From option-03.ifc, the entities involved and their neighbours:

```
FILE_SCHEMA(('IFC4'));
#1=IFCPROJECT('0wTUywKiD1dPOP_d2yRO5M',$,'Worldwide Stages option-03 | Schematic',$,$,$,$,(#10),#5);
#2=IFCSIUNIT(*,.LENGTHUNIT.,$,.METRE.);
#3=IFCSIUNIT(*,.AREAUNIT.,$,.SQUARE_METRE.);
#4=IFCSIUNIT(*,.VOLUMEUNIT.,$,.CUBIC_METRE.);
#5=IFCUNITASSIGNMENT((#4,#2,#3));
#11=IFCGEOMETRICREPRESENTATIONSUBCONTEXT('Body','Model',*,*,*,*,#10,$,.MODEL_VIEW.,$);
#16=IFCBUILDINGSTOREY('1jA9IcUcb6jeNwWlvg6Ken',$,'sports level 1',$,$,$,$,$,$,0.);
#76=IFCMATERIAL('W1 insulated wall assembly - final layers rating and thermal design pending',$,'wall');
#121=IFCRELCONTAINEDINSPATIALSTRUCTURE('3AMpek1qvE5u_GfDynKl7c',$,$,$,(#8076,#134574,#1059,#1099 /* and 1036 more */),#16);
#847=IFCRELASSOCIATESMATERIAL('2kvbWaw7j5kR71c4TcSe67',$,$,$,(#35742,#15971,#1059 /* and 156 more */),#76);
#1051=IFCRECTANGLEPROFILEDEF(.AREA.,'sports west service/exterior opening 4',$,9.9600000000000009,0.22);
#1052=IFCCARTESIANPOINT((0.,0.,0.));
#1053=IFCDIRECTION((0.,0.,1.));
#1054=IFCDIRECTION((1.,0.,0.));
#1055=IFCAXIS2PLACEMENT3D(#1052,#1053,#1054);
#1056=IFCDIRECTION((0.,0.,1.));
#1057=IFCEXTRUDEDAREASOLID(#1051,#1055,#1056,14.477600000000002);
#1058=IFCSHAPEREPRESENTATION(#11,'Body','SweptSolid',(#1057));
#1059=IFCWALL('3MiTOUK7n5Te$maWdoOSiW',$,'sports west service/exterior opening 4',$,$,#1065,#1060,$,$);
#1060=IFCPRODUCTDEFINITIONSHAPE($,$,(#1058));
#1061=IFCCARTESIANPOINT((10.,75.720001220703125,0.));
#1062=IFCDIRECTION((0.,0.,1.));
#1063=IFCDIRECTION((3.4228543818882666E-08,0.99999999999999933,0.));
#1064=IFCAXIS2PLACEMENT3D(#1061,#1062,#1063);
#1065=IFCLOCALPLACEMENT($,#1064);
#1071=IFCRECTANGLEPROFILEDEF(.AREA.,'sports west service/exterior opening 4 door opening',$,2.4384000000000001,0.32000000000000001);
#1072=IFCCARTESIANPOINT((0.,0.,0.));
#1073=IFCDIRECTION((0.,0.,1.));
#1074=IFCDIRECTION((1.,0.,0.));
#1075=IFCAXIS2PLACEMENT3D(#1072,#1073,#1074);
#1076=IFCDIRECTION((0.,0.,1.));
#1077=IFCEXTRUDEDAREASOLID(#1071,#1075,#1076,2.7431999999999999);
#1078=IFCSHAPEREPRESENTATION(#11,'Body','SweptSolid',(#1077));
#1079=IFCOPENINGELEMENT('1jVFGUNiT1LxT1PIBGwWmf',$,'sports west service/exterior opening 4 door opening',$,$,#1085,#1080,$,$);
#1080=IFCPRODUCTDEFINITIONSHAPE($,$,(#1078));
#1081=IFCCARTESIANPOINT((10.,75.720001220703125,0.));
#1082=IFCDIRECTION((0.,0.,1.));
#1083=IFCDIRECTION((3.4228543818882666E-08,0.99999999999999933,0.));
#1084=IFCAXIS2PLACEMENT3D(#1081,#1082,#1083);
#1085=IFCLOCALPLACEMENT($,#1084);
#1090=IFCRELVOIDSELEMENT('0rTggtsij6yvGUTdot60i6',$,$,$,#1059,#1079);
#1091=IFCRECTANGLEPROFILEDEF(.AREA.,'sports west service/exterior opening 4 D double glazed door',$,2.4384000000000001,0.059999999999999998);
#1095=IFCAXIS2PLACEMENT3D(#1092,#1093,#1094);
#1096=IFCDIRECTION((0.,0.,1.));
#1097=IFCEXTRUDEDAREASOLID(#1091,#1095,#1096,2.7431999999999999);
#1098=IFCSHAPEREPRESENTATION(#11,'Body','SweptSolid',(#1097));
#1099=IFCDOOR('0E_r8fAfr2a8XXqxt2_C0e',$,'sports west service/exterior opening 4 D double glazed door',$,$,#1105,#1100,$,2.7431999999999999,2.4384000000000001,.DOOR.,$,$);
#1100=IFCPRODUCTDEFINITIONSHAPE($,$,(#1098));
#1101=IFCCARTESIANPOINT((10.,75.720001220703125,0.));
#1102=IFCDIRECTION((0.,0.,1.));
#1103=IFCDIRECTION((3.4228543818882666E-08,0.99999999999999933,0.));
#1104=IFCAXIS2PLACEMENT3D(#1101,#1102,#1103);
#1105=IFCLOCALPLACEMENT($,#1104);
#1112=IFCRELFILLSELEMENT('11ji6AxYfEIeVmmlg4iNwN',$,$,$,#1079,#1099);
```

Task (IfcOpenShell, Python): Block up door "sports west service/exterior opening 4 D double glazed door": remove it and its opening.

```python
import ifcopenshell
import ifcopenshell.api.feature
import ifcopenshell.api.root
import ifcopenshell.geom
import ifcopenshell.util.shape

model = ifcopenshell.open("option-03.ifc")
settings = ifcopenshell.geom.settings()


def volume(element):
    """Net volume in cubic metres, openings subtracted."""
    shape = ifcopenshell.geom.create_shape(settings, element)
    return ifcopenshell.util.shape.get_volume(shape.geometry)


door = model.by_guid("0E_r8fAfr2a8XXqxt2_C0e")
opening = door.FillsVoids[0].RelatingOpeningElement
wall = opening.VoidsElements[0].RelatingBuildingElement
before = volume(wall)

ifcopenshell.api.root.remove_product(model, product=door)
ifcopenshell.api.feature.remove_feature(model, feature=opening)

after = volume(wall)

print(f"wall volume {before:.3f} -> {after:.3f} m3")

model.write("option-03-out.ifc")
```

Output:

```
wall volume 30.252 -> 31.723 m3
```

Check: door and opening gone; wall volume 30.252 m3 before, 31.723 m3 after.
